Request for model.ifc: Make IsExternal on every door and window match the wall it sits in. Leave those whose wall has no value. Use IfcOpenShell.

First a look at what the model holds.

```python
import ifcopenshell
import ifcopenshell.util.element

model = ifcopenshell.open("model.ifc")
print(model.schema)
seen = {}
for e in model.by_type("IfcDoor") + model.by_type("IfcWindow"):
    if not e.FillsVoids:
        continue
    host = e.FillsVoids[0].RelatingOpeningElement.VoidsElements[0].RelatingBuildingElement
    own = ifcopenshell.util.element.get_pset(e, f"Pset_{e.is_a()[3:].removesuffix('StandardCase')}Common", "IsExternal")
    wall = ifcopenshell.util.element.get_pset(host, "Pset_WallCommon", "IsExternal")
    seen[e.is_a(), own, wall] = seen.get((e.is_a(), own, wall), 0) + 1
for (cls, own, wall), count in sorted(seen.items(), key=str):
    print(count, cls, "IsExternal:", own, "| host wall:", wall)
```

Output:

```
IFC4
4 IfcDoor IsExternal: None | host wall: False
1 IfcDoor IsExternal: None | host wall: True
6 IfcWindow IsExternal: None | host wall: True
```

```python
import ifcopenshell
import ifcopenshell.api.pset
import ifcopenshell.util.element

model = ifcopenshell.open("model.ifc")

count = 0
for ifc_class, pset_name in (("IfcDoor", "Pset_DoorCommon"), ("IfcWindow", "Pset_WindowCommon")):
    for e in model.by_type(ifc_class):
        if not e.FillsVoids:
            continue
        host = e.FillsVoids[0].RelatingOpeningElement.VoidsElements[0].RelatingBuildingElement
        external = ifcopenshell.util.element.get_pset(host, "Pset_WallCommon", "IsExternal")
        if external is None or ifcopenshell.util.element.get_pset(e, pset_name, "IsExternal") == external:
            continue
        pset = ifcopenshell.api.pset.add_pset(model, product=e, name=pset_name)
        ifcopenshell.api.pset.edit_pset(model, pset=pset, properties={"IsExternal": external})
        count += 1

print(count, "updated")

model.write("model-out.ifc")
```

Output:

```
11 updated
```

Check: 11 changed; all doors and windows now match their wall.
